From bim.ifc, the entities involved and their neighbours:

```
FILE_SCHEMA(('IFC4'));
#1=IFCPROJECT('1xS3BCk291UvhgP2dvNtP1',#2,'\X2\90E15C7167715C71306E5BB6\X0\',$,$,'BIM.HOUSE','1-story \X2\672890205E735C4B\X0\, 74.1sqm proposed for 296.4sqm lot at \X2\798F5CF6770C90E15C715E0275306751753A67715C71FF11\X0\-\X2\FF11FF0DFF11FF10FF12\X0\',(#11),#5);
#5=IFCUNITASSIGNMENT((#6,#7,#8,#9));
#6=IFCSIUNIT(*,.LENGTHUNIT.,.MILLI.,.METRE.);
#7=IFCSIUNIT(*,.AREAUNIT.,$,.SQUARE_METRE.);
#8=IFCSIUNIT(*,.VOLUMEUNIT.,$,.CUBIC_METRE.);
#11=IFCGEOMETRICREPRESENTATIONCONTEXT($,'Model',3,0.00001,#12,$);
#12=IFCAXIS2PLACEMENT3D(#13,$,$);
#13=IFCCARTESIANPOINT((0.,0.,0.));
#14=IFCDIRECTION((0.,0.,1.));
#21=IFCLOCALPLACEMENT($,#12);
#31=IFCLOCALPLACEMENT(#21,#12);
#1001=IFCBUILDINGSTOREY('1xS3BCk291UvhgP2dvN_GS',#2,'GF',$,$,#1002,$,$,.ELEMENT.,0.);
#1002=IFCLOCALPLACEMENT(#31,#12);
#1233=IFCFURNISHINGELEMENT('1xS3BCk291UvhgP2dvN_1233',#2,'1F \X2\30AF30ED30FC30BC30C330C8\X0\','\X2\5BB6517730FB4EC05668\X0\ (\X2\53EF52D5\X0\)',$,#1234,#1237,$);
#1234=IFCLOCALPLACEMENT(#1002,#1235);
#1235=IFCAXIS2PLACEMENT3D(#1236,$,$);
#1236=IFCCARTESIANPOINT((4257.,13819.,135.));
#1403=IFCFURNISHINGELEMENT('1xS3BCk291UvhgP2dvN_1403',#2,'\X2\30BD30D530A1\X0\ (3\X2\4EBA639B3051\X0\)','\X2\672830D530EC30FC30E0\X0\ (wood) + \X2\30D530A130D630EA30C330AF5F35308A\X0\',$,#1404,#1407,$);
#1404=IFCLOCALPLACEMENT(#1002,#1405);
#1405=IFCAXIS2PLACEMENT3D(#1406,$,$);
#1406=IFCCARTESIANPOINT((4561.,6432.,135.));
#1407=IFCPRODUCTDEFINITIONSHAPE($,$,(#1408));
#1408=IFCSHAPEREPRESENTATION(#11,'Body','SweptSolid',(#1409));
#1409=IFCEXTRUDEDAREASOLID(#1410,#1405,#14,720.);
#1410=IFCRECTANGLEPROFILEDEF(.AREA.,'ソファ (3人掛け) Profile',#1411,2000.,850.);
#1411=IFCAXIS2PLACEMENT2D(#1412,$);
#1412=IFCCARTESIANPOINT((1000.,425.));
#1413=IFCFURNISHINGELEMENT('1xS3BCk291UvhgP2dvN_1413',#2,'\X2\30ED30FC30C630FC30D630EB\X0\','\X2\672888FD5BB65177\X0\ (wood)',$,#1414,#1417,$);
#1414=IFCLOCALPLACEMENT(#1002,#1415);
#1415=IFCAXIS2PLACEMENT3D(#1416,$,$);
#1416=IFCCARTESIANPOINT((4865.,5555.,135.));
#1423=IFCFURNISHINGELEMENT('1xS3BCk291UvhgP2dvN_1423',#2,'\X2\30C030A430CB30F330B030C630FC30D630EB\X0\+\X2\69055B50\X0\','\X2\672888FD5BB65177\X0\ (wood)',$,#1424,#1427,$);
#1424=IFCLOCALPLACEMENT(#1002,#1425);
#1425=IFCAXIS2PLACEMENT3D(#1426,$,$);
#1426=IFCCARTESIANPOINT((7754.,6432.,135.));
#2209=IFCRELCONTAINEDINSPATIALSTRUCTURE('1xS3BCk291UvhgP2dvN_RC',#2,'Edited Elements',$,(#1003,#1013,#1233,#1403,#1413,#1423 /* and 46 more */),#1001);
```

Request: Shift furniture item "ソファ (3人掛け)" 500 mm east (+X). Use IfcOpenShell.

```python
import ifcopenshell
import ifcopenshell.api.geometry
import ifcopenshell.util.placement

model = ifcopenshell.open("bim.ifc")

item = model.by_guid("1xS3BCk291UvhgP2dvN_1403")
matrix = ifcopenshell.util.placement.get_local_placement(item.ObjectPlacement)
matrix[0, 3] += 500.0
ifcopenshell.api.geometry.edit_object_placement(model, product=item, matrix=matrix, is_si=False)

print(ifcopenshell.util.placement.get_local_placement(item.ObjectPlacement).round(3) + 0.0)

model.write("bim_rev.ifc")
```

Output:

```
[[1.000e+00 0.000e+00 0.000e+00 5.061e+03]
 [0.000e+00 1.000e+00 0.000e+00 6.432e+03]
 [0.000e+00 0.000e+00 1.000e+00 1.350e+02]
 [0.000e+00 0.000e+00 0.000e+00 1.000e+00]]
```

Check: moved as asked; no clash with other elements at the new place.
